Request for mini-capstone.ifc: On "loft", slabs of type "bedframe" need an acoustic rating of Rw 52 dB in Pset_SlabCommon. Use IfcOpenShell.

First a look at what the model holds.

```python
import ifcopenshell
import ifcopenshell.util.element

model = ifcopenshell.open("mini-capstone.ifc")
print(model.schema)
storey = next(s for s in model.by_type("IfcBuildingStorey") if s.Name == "loft")
slabs = [e for e in ifcopenshell.util.element.get_decomposition(storey) if e.is_a("IfcSlab")]
seen = {}
for e in slabs:
    element_type = ifcopenshell.util.element.get_type(e)
    key = (element_type.Name if element_type != e and element_type else None, ifcopenshell.util.element.get_pset(e, "Pset_SlabCommon", "AcousticRating"))
    seen[key] = seen.get(key, 0) + 1
for (name, value), count in sorted(seen.items(), key=str):
    print(count, "x", name, "|", value)
```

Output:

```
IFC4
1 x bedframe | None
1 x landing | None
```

```python
import ifcopenshell
import ifcopenshell.api.pset
import ifcopenshell.util.element

model = ifcopenshell.open("mini-capstone.ifc")

storey = next(s for s in model.by_type("IfcBuildingStorey") if s.Name == "loft")
slabs = [e for e in ifcopenshell.util.element.get_decomposition(storey) if e.is_a("IfcSlab")]

count = 0
for e in slabs:
    element_type = ifcopenshell.util.element.get_type(e)
    if element_type in (None, e) or element_type.Name != "bedframe":
        continue
    # add_pset returns the element's existing set when there is one.
    pset = ifcopenshell.api.pset.add_pset(model, product=e, name="Pset_SlabCommon")
    ifcopenshell.api.pset.edit_pset(model, pset=pset, properties={"AcousticRating": "Rw 52 dB"})
    count += 1

print(count, "slabs updated")

model.write("mini-capstone-out.ifc")
```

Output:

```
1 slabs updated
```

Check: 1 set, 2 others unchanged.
